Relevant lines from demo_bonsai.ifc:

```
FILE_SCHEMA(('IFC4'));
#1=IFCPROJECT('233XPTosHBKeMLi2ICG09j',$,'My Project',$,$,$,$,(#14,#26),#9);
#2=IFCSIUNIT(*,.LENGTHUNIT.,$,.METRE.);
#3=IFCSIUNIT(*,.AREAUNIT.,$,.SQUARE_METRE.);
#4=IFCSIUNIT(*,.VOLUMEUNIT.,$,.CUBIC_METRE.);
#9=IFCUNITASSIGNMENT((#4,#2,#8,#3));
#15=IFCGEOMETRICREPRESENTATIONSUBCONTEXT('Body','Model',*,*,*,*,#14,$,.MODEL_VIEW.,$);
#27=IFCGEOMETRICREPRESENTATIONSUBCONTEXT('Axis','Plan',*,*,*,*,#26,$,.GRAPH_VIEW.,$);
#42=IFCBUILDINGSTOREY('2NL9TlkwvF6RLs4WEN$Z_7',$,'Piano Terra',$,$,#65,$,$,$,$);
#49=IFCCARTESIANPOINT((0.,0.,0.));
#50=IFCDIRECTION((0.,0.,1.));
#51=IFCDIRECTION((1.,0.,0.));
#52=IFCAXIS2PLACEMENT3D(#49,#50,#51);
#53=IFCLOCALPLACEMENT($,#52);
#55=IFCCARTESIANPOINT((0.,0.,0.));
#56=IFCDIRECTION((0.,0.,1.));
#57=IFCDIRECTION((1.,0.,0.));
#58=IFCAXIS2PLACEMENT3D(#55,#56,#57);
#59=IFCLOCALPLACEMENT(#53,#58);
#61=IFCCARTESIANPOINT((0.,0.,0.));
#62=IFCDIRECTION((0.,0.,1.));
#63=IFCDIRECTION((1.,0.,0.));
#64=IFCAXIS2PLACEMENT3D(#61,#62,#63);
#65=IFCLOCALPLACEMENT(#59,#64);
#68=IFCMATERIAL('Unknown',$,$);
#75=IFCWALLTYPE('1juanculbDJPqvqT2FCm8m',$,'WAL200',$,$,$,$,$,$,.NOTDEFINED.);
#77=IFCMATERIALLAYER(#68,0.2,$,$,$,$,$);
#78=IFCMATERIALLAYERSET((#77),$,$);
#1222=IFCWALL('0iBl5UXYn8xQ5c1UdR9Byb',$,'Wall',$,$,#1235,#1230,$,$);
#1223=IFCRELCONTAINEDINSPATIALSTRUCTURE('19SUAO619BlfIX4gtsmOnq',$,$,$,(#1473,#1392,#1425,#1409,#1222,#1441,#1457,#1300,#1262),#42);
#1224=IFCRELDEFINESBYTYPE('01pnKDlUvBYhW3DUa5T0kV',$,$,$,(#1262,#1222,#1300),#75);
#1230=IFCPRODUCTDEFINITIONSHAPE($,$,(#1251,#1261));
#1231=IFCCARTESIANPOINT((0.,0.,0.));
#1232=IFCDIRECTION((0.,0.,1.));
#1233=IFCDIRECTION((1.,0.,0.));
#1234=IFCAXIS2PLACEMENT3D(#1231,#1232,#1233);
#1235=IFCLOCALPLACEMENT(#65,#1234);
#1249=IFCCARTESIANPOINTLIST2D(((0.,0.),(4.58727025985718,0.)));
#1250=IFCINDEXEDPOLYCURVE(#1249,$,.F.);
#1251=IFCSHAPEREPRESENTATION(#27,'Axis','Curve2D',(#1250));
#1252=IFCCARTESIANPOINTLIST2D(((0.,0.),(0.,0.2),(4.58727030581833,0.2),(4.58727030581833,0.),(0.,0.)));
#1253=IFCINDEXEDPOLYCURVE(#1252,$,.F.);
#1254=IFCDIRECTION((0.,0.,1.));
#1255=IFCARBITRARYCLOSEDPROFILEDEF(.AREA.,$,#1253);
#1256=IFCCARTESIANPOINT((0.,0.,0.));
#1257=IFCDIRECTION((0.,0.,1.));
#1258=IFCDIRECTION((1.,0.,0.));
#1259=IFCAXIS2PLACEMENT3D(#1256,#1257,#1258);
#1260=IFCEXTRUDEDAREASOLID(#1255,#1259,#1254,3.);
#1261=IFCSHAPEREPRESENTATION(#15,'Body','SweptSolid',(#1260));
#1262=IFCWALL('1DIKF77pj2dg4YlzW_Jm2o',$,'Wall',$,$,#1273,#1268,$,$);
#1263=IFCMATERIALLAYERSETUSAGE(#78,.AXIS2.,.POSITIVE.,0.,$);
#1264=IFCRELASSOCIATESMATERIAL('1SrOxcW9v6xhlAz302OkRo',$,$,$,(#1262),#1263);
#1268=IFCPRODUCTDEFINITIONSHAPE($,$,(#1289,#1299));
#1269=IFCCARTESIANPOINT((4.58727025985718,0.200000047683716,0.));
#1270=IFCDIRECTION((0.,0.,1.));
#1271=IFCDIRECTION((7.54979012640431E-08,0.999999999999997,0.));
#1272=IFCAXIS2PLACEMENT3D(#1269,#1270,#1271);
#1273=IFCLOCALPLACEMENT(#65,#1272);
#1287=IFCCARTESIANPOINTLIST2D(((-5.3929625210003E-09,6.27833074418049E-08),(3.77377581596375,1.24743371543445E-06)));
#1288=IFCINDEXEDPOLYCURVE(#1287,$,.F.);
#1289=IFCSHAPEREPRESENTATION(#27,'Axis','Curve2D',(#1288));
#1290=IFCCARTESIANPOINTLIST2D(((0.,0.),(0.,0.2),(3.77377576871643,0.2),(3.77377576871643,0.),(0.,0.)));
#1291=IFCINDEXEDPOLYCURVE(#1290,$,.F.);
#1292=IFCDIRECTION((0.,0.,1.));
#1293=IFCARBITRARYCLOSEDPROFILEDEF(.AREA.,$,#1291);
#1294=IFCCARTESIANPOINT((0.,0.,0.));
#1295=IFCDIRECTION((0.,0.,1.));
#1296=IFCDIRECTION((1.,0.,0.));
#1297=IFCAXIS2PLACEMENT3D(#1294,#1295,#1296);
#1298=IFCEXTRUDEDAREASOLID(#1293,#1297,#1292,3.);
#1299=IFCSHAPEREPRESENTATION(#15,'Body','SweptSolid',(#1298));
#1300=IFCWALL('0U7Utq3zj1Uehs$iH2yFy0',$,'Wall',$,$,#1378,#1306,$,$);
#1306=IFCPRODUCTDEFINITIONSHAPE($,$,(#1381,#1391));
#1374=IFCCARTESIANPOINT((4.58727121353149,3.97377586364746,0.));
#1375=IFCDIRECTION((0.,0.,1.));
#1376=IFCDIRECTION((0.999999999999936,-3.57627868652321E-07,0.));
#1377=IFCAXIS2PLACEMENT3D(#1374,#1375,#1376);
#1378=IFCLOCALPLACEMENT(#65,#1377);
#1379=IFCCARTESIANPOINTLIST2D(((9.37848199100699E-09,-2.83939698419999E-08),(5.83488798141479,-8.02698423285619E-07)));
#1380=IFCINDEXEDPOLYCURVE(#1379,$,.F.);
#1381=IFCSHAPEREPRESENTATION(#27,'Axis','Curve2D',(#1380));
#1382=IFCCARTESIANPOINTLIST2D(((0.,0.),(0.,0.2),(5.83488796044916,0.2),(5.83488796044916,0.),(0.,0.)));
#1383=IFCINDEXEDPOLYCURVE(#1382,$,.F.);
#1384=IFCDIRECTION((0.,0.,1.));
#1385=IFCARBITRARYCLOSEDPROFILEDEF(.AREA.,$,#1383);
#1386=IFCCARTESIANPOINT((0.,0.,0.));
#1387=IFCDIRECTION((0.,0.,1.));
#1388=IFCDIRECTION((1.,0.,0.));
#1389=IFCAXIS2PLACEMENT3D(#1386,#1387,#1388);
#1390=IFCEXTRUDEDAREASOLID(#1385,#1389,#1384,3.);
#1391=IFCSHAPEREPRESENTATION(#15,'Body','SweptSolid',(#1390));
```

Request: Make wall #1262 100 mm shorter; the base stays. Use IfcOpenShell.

```python
import ifcopenshell
import ifcopenshell.geom
import ifcopenshell.util.representation
import ifcopenshell.util.shape
import ifcopenshell.util.unit

model = ifcopenshell.open("demo_bonsai.ifc")
unit_scale = ifcopenshell.util.unit.calculate_unit_scale(model)
settings = ifcopenshell.geom.settings()


def volume(element):
    """Net volume in cubic metres, openings subtracted."""
    shape = ifcopenshell.geom.create_shape(settings, element)
    return ifcopenshell.util.shape.get_volume(shape.geometry)


wall = model.by_guid("1DIKF77pj2dg4YlzW_Jm2o")
before = volume(wall)

body = ifcopenshell.util.representation.get_representation(wall, "Model", "Body")
solid = body.Items[0]
old_height = solid.Depth
solid.Depth -= 0.1 / unit_scale
after = volume(wall)

print(f"height {old_height:g} -> {solid.Depth:g}, volume {before:.3f} -> {after:.3f} m3")

model.write("demo_bonsai_rev.ifc")
```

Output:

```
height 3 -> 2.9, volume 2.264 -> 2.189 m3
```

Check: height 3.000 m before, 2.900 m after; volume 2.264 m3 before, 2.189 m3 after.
